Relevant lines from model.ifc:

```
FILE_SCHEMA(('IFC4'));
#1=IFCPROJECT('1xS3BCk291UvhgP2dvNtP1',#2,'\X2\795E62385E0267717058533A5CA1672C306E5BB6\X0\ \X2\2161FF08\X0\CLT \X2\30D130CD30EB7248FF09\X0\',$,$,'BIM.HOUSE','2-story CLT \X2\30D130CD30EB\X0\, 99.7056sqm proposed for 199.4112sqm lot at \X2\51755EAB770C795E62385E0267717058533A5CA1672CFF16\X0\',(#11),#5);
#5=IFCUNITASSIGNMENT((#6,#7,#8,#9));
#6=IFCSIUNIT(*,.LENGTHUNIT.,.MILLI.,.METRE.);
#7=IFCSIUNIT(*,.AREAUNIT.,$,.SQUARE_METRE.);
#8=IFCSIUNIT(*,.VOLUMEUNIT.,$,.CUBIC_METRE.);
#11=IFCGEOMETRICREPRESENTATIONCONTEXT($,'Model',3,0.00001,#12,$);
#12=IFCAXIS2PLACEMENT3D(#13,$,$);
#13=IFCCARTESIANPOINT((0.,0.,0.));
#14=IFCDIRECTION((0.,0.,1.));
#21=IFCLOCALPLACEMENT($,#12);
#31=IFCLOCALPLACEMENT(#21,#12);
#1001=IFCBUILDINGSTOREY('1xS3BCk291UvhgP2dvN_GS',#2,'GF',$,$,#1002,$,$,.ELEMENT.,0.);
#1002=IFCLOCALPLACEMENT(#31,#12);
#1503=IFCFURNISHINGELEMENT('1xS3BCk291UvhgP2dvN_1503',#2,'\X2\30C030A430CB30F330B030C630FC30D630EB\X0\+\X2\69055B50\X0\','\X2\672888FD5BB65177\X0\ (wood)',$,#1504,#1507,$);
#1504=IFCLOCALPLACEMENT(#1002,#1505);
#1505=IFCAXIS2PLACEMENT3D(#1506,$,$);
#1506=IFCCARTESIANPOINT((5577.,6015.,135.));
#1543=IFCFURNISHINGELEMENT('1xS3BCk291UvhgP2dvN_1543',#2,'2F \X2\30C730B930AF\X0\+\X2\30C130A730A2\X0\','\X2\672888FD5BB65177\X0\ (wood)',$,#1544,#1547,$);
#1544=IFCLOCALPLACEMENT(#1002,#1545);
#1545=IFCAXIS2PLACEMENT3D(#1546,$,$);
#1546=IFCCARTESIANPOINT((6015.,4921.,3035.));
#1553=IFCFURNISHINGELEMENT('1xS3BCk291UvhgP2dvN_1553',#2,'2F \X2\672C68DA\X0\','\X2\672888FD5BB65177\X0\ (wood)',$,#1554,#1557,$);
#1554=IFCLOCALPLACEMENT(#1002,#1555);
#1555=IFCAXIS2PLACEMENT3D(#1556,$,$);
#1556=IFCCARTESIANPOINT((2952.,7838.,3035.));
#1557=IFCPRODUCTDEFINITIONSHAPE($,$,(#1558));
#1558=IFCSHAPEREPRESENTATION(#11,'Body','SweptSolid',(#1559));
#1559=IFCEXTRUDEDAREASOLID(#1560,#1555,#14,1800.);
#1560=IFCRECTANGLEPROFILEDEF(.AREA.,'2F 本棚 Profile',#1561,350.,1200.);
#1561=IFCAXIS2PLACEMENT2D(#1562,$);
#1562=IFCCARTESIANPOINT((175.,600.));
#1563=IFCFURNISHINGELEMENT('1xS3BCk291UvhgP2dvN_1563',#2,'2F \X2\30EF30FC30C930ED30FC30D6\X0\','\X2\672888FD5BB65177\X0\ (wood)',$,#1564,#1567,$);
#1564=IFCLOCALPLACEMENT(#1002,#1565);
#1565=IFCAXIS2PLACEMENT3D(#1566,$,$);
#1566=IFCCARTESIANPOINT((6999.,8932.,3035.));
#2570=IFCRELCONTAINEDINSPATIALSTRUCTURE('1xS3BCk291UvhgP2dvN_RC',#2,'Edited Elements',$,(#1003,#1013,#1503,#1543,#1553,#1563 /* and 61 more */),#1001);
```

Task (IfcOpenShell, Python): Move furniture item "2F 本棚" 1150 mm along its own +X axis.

```python
import ifcopenshell
import ifcopenshell.api.geometry
import ifcopenshell.util.placement
import ifcopenshell.util.unit

model = ifcopenshell.open("model.ifc")
unit_scale = ifcopenshell.util.unit.calculate_unit_scale(model)

item = model.by_id(1553)
matrix = ifcopenshell.util.placement.get_local_placement(item.ObjectPlacement)
matrix[:3, 3] += matrix[:3, 0] * 1.15 / unit_scale
ifcopenshell.api.geometry.edit_object_placement(model, product=item, matrix=matrix, is_si=False)

print(ifcopenshell.util.placement.get_local_placement(item.ObjectPlacement).round(3) + 0.0)

model.write("model_edited.ifc")
```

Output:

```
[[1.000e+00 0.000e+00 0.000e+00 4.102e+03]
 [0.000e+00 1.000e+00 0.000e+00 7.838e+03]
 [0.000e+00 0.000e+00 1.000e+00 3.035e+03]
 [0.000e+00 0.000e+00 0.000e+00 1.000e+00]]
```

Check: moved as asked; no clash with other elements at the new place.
